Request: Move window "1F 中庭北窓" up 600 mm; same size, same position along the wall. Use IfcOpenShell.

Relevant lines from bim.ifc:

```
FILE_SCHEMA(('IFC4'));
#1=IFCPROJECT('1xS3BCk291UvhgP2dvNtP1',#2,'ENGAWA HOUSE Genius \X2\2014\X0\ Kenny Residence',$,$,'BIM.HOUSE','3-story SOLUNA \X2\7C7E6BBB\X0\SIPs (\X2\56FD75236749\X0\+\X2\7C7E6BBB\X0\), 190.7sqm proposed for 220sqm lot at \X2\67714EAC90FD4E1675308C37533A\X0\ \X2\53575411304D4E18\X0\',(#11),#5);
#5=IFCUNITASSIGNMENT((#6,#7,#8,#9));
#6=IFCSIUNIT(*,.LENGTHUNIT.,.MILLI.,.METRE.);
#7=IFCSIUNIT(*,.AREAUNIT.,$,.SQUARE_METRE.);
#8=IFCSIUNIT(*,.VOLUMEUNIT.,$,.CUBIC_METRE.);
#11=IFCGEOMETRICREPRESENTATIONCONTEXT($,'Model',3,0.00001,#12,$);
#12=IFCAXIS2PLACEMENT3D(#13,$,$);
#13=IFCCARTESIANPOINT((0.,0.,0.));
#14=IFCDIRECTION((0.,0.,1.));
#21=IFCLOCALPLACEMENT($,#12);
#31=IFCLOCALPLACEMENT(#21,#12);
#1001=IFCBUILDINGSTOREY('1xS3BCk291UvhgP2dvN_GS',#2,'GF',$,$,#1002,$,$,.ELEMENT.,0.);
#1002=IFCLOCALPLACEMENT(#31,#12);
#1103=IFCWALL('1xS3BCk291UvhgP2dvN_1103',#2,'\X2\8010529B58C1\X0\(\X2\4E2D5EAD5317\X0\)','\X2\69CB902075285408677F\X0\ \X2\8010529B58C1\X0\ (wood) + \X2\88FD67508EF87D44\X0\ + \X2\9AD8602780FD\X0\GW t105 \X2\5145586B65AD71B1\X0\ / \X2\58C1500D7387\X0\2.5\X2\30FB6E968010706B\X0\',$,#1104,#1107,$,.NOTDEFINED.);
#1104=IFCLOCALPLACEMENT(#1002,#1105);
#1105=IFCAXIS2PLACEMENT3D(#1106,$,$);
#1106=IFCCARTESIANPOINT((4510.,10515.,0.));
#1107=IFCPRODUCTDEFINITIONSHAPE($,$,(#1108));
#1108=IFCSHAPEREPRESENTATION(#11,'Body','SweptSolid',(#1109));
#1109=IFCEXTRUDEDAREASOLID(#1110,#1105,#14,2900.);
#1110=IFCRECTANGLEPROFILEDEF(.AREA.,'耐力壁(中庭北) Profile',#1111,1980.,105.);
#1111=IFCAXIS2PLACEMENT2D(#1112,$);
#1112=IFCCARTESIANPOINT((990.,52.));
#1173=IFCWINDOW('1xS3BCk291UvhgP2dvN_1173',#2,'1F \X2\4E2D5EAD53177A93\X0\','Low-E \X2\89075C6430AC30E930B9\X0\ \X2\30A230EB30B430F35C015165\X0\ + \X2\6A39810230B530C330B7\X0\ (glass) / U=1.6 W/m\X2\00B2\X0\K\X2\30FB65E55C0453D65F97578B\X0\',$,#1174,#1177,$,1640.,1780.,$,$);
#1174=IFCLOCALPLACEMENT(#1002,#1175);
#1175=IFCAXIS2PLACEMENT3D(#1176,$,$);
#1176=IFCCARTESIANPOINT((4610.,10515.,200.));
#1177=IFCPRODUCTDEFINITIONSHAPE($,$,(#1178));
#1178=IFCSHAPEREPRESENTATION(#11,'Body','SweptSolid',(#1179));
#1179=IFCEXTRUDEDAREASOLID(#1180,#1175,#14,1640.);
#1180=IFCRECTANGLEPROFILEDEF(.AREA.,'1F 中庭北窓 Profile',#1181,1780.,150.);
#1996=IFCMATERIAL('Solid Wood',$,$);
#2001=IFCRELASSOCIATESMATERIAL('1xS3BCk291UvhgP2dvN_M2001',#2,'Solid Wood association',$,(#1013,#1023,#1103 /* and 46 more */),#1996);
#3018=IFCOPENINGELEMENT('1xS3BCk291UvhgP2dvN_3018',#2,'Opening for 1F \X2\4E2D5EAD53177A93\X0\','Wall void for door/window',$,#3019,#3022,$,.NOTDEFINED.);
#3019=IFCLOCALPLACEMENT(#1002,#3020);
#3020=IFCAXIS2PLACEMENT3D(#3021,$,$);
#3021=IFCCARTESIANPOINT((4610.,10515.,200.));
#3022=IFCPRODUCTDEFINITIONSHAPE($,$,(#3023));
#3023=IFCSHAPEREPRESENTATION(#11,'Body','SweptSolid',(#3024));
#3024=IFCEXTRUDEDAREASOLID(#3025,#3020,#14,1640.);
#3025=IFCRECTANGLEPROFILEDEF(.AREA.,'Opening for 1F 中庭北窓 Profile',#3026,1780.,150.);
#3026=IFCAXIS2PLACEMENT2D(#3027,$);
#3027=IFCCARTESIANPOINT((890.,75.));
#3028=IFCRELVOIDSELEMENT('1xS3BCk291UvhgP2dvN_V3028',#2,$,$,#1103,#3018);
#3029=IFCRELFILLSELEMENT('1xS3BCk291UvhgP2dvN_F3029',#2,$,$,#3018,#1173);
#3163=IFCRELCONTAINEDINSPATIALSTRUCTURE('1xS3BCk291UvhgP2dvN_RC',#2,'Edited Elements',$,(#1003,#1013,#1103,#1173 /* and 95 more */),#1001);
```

```python
import numpy as np
import ifcopenshell
import ifcopenshell.api.geometry
import ifcopenshell.util.placement
import ifcopenshell.util.unit

model = ifcopenshell.open("bim.ifc")
unit_scale = ifcopenshell.util.unit.calculate_unit_scale(model)

window = model.by_guid("1xS3BCk291UvhgP2dvN_1173")
opening = window.FillsVoids[0].RelatingOpeningElement
dz = 600.0

shift = np.array([0.0, 0.0, dz])
# The window is not placed relative to its opening, so move both.
for product in (opening, window):
    matrix = ifcopenshell.util.placement.get_local_placement(product.ObjectPlacement)
    matrix[:3, 3] += shift
    ifcopenshell.api.geometry.edit_object_placement(model, product=product, matrix=matrix, is_si=False)

print(f"moved by {dz * unit_scale:+.3f} m")

model.write("bim_rev.ifc")
```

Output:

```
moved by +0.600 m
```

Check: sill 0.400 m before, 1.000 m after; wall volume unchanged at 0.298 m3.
